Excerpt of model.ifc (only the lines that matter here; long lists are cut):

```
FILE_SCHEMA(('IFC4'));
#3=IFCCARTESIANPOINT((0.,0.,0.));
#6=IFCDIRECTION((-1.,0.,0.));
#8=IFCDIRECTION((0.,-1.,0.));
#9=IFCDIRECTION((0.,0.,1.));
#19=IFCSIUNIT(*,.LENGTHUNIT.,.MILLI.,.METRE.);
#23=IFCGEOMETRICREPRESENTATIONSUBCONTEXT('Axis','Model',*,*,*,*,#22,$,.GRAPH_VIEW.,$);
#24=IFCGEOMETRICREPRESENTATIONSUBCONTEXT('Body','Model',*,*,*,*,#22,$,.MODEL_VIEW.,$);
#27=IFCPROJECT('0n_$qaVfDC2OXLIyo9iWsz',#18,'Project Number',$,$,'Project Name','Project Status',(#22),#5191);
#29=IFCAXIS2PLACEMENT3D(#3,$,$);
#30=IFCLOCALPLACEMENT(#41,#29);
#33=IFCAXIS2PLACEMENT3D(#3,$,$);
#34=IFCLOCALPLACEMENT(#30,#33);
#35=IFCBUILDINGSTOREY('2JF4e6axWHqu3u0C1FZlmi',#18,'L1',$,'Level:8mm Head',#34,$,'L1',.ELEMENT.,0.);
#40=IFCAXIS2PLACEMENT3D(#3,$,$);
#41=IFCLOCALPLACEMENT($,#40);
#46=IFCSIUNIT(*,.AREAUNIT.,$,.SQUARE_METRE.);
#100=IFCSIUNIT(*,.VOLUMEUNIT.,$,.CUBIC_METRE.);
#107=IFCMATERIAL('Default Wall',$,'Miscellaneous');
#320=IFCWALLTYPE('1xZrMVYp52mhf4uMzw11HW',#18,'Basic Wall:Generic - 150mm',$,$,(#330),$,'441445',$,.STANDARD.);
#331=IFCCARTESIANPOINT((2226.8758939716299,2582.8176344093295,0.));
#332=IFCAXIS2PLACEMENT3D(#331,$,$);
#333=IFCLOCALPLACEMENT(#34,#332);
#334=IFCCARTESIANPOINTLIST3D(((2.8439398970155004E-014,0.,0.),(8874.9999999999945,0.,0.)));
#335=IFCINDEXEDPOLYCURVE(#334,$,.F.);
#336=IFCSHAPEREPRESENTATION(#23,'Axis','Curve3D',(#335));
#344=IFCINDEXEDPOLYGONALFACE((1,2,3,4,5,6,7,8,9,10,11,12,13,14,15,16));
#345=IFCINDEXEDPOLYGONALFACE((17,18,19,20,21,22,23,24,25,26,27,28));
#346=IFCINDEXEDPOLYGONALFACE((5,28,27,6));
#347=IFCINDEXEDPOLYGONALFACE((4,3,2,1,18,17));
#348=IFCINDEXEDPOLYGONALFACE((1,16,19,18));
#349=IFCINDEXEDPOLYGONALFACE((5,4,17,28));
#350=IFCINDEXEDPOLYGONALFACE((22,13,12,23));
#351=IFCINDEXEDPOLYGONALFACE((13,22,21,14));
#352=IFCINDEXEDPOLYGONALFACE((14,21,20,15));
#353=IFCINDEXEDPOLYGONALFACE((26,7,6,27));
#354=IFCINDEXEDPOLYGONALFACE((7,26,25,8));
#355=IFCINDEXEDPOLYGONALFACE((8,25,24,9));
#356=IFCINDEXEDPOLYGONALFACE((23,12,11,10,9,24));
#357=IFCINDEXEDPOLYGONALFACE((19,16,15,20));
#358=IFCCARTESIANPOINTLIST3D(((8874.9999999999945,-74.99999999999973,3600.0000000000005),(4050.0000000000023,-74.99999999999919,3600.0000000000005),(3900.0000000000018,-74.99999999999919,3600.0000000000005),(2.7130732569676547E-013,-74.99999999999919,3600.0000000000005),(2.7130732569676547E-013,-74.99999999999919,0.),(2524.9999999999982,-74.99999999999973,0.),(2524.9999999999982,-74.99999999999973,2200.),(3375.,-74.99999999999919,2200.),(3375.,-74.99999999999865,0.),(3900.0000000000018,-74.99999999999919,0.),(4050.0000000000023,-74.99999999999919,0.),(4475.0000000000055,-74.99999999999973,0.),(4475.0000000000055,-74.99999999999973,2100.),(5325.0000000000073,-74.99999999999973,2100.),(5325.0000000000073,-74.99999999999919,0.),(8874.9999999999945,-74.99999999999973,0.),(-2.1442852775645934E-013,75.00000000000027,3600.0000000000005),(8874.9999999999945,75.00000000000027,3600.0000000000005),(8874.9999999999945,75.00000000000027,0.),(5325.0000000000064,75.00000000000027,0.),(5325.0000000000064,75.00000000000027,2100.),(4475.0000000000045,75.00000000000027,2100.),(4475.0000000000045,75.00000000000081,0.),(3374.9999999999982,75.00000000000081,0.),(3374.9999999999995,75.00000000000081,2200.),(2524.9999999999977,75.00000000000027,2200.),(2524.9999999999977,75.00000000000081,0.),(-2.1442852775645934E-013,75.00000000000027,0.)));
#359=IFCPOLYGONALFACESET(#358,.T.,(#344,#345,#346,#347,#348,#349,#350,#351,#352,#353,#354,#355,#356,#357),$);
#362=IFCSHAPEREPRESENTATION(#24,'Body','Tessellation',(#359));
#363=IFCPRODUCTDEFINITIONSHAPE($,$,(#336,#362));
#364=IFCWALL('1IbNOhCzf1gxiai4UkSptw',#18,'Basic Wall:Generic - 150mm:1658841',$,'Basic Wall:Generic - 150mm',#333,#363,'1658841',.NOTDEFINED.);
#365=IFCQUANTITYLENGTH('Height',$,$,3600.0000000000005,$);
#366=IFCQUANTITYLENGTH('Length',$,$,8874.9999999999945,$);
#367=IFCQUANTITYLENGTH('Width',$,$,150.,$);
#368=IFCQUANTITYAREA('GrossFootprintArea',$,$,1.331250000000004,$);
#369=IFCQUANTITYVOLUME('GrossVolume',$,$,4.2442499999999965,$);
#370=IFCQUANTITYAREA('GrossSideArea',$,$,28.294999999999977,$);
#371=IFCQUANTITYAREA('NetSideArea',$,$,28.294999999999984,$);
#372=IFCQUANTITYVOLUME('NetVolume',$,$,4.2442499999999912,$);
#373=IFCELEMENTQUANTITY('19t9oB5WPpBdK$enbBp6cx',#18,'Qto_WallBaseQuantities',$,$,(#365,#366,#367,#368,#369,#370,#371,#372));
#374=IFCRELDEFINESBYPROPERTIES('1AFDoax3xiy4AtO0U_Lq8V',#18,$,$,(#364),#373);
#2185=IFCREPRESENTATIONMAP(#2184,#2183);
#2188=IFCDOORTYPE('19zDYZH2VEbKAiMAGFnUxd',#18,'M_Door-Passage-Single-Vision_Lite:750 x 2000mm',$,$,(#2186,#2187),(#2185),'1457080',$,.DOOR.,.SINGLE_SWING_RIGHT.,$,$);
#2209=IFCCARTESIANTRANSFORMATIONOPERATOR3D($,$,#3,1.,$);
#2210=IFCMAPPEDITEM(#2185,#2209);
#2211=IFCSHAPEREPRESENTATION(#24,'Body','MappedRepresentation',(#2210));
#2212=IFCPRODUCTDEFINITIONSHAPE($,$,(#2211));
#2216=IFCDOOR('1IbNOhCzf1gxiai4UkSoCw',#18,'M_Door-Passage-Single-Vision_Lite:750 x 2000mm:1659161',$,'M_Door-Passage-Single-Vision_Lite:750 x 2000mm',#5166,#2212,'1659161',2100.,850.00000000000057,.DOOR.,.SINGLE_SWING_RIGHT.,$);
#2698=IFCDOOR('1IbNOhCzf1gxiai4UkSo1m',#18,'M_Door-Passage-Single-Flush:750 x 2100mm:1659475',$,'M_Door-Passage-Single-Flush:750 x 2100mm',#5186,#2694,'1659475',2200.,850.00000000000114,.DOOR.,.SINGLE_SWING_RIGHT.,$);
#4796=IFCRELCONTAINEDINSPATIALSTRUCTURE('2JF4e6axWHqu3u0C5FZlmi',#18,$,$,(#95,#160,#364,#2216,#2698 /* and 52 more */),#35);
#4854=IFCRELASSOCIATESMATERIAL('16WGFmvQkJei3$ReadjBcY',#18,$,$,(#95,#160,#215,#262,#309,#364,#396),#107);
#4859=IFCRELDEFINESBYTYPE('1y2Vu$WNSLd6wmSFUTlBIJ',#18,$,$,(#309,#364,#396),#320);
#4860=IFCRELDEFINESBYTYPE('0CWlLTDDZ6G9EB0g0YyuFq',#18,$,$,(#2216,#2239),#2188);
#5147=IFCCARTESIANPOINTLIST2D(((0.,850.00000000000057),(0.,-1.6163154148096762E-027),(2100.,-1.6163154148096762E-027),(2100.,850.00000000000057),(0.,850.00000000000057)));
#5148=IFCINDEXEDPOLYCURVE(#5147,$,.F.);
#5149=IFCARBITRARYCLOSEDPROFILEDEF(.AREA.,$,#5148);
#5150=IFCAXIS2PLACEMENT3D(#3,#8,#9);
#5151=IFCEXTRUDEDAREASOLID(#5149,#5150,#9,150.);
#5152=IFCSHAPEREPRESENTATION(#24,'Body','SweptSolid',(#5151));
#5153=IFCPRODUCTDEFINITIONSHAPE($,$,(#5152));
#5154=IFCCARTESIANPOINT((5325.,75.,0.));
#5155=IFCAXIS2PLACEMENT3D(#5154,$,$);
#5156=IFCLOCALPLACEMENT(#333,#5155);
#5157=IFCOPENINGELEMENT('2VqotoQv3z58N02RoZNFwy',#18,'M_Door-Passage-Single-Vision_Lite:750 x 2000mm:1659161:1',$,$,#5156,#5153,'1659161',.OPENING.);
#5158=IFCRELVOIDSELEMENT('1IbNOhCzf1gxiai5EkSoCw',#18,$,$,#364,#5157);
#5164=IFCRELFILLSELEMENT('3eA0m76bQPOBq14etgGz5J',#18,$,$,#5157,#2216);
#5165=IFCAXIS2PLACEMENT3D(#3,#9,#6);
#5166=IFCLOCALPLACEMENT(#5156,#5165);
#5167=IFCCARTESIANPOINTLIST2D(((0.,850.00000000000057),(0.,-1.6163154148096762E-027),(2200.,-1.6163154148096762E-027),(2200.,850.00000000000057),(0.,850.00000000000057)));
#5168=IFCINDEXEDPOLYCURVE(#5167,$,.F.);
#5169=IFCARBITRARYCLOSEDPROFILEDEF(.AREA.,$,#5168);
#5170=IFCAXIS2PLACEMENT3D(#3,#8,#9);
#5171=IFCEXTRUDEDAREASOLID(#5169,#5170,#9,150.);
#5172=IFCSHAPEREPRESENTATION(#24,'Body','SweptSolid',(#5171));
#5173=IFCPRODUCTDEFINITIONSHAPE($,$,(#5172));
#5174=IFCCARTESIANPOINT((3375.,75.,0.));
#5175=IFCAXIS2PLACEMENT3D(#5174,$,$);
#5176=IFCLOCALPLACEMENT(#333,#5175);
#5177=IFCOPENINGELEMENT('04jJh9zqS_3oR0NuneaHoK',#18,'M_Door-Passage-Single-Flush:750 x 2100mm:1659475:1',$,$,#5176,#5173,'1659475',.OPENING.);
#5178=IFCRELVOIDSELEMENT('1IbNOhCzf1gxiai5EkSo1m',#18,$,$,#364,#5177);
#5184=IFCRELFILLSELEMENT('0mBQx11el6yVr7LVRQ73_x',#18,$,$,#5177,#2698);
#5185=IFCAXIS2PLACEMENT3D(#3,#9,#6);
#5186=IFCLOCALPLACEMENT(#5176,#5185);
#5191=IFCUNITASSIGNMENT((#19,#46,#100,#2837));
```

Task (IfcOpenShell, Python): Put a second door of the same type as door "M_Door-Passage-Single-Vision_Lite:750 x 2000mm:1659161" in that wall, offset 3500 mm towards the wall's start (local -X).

```python
import ifcopenshell
import ifcopenshell.api.feature
import ifcopenshell.api.geometry
import ifcopenshell.api.pset
import ifcopenshell.api.root
import ifcopenshell.geom
import ifcopenshell.util.element
import ifcopenshell.util.placement
import ifcopenshell.util.shape
import ifcopenshell.util.unit

model = ifcopenshell.open("model.ifc")
unit_scale = ifcopenshell.util.unit.calculate_unit_scale(model)
area_scale = ifcopenshell.util.unit.calculate_unit_scale(model, "AREAUNIT")
volume_scale = ifcopenshell.util.unit.calculate_unit_scale(model, "VOLUMEUNIT")
settings = ifcopenshell.geom.settings()


def volume(element):
    """Net volume in cubic metres, openings subtracted."""
    shape = ifcopenshell.geom.create_shape(settings, element)
    return ifcopenshell.util.shape.get_volume(shape.geometry)


def reuse_history(source, copy):
    """copy_class also copies each property set's owner history, people and application; keep the originals."""
    for rel in copy.IsDefinedBy:
        if rel.is_a("IfcRelDefinesByProperties") and (history := rel.RelatingPropertyDefinition.OwnerHistory):
            rel.RelatingPropertyDefinition.OwnerHistory = source.OwnerHistory
            ifcopenshell.util.element.remove_deep2(model, history)


door = model.by_guid("1IbNOhCzf1gxiai4UkSoCw")
opening = door.FillsVoids[0].RelatingOpeningElement
wall = opening.VoidsElements[0].RelatingBuildingElement
before = volume(wall)
shift = ifcopenshell.util.placement.get_local_placement(wall.ObjectPlacement)[:3, 0] * -3.5 / unit_scale

# copy_class copies the void relationship, type, container and properties, but no geometry.
new_opening = ifcopenshell.api.root.copy_class(model, product=opening)
new_opening.Representation = ifcopenshell.util.element.copy_deep(
    model, opening.Representation, exclude=["IfcGeometricRepresentationContext", "IfcRepresentationMap"]
)
new_opening.Name = "M_Door-Passage-Single-Vision_Lite:750 x 2000mm"
new_opening.Tag = None
reuse_history(opening, new_opening)
new_door = ifcopenshell.api.root.copy_class(model, product=door)
new_door.Representation = ifcopenshell.util.element.copy_deep(
    model, door.Representation, exclude=["IfcGeometricRepresentationContext", "IfcRepresentationMap"]
)
new_door.Name = "M_Door-Passage-Single-Vision_Lite:750 x 2000mm"
new_door.Tag = None
reuse_history(door, new_door)
ifcopenshell.api.feature.add_filling(model, opening=new_opening, element=new_door)

for old, new in ((opening, new_opening), (door, new_door)):
    matrix = ifcopenshell.util.placement.get_local_placement(old.ObjectPlacement)
    matrix[:3, 3] += shift
    ifcopenshell.api.geometry.edit_object_placement(model, product=new, matrix=matrix, is_si=False)

after = volume(wall)
thickness = 0.15  # wall thickness in metres

# Update the wall's stored quantities.
qto = model.by_id(ifcopenshell.util.element.get_pset(wall, "Qto_WallBaseQuantities", should_inherit=False)["id"])
ifcopenshell.api.pset.edit_qto(model, qto=qto, properties={
    "NetSideArea": after / thickness / area_scale,
    "NetVolume": after / volume_scale,
})

print(f"wall volume {before:.3f} -> {after:.3f} m3")

model.write("model_rev.ifc")
```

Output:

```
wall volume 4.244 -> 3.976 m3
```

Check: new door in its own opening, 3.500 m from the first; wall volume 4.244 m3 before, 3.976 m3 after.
